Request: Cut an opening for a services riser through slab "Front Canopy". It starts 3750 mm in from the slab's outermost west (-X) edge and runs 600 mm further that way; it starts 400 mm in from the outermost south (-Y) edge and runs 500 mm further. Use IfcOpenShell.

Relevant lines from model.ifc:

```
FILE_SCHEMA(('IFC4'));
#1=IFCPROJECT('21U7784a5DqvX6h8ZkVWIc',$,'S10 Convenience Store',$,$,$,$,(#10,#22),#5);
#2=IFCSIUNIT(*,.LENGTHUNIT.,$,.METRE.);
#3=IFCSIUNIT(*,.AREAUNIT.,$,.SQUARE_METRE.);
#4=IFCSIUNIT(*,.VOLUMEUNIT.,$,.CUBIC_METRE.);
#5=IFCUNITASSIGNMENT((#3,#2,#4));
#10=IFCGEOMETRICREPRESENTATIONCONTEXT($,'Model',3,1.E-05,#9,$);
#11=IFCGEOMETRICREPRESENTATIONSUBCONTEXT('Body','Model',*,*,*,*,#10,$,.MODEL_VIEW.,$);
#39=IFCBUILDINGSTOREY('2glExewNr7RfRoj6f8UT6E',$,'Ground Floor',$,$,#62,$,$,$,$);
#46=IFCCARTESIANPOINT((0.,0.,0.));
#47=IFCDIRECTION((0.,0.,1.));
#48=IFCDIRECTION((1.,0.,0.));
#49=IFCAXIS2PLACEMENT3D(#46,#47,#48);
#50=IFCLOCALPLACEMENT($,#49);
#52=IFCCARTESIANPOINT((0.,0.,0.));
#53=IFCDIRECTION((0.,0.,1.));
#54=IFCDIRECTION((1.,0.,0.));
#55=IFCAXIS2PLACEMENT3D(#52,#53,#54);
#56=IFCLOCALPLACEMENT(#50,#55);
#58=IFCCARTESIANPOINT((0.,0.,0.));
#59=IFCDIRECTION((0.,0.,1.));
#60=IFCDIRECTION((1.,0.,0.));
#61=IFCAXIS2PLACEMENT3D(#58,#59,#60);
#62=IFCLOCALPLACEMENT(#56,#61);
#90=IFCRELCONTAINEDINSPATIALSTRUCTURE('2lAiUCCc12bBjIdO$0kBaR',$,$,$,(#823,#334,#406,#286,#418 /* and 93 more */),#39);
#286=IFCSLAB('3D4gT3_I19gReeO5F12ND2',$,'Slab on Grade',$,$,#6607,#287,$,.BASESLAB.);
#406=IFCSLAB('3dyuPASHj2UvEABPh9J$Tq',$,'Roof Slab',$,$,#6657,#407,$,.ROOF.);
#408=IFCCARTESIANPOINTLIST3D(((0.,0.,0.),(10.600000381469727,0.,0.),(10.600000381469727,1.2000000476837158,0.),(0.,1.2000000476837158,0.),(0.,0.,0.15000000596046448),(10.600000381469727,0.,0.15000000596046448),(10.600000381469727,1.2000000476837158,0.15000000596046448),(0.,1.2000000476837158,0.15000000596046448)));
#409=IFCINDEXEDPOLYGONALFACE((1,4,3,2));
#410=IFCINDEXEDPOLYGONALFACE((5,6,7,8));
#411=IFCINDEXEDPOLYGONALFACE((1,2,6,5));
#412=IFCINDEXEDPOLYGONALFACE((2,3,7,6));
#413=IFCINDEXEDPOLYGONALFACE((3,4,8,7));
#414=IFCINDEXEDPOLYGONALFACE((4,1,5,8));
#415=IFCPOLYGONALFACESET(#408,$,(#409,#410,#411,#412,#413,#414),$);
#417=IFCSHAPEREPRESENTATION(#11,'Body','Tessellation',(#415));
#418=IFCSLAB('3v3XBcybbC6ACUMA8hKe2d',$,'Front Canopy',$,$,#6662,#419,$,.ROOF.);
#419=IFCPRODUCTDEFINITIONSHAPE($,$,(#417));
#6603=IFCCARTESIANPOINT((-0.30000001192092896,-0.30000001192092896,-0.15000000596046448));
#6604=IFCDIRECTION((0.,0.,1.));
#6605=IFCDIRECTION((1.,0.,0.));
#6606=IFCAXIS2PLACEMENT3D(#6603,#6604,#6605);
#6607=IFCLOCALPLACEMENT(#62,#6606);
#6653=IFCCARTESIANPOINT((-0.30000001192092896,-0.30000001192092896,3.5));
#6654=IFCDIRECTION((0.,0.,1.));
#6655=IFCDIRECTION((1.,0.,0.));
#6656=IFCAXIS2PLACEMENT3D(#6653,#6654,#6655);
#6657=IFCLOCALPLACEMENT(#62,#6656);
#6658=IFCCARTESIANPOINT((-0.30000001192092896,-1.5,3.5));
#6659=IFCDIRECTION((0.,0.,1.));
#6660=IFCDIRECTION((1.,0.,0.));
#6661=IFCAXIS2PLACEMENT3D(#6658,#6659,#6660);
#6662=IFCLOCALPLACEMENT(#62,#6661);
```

```python
import numpy as np
import ifcopenshell
import ifcopenshell.api.feature
import ifcopenshell.api.geometry
import ifcopenshell.api.root
import ifcopenshell.geom
import ifcopenshell.util.placement
import ifcopenshell.util.representation
import ifcopenshell.util.shape
import ifcopenshell.util.unit

model = ifcopenshell.open("model.ifc")
unit_scale = ifcopenshell.util.unit.calculate_unit_scale(model)
settings = ifcopenshell.geom.settings()


def volume(element):
    """Net volume in cubic metres, openings subtracted."""
    shape = ifcopenshell.geom.create_shape(settings, element)
    return ifcopenshell.util.shape.get_volume(shape.geometry)


slab = model.by_guid("3v3XBcybbC6ACUMA8hKe2d")
before = volume(slab)

# Extent in the slab's own axes, in metres. The edges named are its -X and -Y sides.
slab_shape = ifcopenshell.geom.create_shape(settings, slab)
vertices = ifcopenshell.util.shape.get_vertices(slab_shape.geometry)
x_min, y_min, bottom = vertices.min(axis=0)
top = vertices[:, 2].max()

opening = ifcopenshell.api.root.create_entity(model, ifc_class="IfcOpeningElement", name="Services riser opening", predefined_type="OPENING")
context = ifcopenshell.util.representation.get_context(model, "Model", "Body", "MODEL_VIEW")
width, depth = 0.6, 0.5
outline = [(0.0, 0.0), (width, 0.0), (width, depth), (0.0, depth), (0.0, 0.0)]
# Overshoot both faces by 50 mm so the cut is clean.
shape = ifcopenshell.api.geometry.add_slab_representation(
    model, context=context, depth=top - bottom + 0.1, polyline=outline
)
ifcopenshell.api.geometry.assign_representation(model, product=opening, representation=shape)

matrix = ifcopenshell.util.placement.get_local_placement(slab.ObjectPlacement)
matrix[:, 3] = matrix @ np.append(np.array([x_min + 3.75, y_min + 0.4, bottom - 0.05]) / unit_scale, 1.0)
ifcopenshell.api.geometry.edit_object_placement(model, product=opening, matrix=matrix, is_si=False)
ifcopenshell.api.feature.add_feature(model, feature=opening, element=slab)

after = volume(slab)

print(f"slab volume {before:.3f} -> {after:.3f} m3")

model.write("model_edited.ifc")
```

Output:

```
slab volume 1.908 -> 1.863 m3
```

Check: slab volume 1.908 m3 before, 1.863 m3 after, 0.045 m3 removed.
